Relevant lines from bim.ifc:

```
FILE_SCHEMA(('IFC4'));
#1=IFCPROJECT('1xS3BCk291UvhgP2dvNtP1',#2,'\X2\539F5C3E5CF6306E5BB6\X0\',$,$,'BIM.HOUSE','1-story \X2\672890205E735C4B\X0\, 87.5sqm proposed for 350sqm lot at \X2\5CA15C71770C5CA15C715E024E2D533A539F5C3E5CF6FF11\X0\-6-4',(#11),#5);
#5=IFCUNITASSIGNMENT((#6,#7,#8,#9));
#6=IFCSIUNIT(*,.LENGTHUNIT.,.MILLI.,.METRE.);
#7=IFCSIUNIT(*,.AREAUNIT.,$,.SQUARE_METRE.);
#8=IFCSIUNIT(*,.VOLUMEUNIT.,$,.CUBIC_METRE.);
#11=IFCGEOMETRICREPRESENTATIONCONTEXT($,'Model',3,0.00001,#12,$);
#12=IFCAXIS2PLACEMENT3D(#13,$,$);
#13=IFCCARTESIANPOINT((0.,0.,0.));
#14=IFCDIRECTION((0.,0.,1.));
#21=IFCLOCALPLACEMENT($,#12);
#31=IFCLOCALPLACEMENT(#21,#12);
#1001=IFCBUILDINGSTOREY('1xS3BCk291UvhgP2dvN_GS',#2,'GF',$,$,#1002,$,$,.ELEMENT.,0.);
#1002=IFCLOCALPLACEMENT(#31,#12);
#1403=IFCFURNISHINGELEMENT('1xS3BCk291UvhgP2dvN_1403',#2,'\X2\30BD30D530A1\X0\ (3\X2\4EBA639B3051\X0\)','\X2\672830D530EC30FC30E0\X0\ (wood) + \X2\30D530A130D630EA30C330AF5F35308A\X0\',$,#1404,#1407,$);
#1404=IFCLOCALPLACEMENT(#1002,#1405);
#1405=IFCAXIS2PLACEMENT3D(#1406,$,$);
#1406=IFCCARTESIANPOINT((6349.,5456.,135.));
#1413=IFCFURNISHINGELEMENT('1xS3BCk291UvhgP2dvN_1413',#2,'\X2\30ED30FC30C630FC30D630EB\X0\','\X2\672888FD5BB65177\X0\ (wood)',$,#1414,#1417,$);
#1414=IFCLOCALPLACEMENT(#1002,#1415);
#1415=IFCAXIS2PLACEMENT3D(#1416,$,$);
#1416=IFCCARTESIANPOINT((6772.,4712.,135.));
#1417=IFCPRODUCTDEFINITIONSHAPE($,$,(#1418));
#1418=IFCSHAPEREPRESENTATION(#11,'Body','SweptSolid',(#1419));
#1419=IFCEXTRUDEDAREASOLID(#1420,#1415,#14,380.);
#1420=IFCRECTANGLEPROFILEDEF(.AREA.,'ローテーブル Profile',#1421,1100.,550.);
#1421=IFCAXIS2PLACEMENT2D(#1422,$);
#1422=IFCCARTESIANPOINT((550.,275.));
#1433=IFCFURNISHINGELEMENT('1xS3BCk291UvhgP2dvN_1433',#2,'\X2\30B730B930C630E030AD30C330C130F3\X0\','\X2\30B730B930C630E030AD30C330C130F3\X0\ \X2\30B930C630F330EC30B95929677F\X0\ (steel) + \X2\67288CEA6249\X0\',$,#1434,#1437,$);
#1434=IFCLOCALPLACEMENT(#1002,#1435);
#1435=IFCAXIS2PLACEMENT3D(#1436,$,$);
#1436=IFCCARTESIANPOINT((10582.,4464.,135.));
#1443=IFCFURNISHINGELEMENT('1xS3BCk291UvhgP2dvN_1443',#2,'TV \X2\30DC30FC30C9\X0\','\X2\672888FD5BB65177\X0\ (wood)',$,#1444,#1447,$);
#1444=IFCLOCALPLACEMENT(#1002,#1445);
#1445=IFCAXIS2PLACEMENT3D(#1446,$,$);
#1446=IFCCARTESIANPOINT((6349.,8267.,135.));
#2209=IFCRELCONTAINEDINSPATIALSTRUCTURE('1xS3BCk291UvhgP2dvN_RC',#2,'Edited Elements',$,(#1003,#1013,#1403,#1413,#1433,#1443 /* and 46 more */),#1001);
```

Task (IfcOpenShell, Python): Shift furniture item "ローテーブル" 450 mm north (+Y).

```python
import ifcopenshell
import ifcopenshell.api.geometry
import ifcopenshell.util.placement

model = ifcopenshell.open("bim.ifc")

item = model.by_guid("1xS3BCk291UvhgP2dvN_1413")
matrix = ifcopenshell.util.placement.get_local_placement(item.ObjectPlacement)
matrix[1, 3] += 450.0
ifcopenshell.api.geometry.edit_object_placement(model, product=item, matrix=matrix, is_si=False)

print(ifcopenshell.util.placement.get_local_placement(item.ObjectPlacement).round(3) + 0.0)

model.write("bim_rev.ifc")
```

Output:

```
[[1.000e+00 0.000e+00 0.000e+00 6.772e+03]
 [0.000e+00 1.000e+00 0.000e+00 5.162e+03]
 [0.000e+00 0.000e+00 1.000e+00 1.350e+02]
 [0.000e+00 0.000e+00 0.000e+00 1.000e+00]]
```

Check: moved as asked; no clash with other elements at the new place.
